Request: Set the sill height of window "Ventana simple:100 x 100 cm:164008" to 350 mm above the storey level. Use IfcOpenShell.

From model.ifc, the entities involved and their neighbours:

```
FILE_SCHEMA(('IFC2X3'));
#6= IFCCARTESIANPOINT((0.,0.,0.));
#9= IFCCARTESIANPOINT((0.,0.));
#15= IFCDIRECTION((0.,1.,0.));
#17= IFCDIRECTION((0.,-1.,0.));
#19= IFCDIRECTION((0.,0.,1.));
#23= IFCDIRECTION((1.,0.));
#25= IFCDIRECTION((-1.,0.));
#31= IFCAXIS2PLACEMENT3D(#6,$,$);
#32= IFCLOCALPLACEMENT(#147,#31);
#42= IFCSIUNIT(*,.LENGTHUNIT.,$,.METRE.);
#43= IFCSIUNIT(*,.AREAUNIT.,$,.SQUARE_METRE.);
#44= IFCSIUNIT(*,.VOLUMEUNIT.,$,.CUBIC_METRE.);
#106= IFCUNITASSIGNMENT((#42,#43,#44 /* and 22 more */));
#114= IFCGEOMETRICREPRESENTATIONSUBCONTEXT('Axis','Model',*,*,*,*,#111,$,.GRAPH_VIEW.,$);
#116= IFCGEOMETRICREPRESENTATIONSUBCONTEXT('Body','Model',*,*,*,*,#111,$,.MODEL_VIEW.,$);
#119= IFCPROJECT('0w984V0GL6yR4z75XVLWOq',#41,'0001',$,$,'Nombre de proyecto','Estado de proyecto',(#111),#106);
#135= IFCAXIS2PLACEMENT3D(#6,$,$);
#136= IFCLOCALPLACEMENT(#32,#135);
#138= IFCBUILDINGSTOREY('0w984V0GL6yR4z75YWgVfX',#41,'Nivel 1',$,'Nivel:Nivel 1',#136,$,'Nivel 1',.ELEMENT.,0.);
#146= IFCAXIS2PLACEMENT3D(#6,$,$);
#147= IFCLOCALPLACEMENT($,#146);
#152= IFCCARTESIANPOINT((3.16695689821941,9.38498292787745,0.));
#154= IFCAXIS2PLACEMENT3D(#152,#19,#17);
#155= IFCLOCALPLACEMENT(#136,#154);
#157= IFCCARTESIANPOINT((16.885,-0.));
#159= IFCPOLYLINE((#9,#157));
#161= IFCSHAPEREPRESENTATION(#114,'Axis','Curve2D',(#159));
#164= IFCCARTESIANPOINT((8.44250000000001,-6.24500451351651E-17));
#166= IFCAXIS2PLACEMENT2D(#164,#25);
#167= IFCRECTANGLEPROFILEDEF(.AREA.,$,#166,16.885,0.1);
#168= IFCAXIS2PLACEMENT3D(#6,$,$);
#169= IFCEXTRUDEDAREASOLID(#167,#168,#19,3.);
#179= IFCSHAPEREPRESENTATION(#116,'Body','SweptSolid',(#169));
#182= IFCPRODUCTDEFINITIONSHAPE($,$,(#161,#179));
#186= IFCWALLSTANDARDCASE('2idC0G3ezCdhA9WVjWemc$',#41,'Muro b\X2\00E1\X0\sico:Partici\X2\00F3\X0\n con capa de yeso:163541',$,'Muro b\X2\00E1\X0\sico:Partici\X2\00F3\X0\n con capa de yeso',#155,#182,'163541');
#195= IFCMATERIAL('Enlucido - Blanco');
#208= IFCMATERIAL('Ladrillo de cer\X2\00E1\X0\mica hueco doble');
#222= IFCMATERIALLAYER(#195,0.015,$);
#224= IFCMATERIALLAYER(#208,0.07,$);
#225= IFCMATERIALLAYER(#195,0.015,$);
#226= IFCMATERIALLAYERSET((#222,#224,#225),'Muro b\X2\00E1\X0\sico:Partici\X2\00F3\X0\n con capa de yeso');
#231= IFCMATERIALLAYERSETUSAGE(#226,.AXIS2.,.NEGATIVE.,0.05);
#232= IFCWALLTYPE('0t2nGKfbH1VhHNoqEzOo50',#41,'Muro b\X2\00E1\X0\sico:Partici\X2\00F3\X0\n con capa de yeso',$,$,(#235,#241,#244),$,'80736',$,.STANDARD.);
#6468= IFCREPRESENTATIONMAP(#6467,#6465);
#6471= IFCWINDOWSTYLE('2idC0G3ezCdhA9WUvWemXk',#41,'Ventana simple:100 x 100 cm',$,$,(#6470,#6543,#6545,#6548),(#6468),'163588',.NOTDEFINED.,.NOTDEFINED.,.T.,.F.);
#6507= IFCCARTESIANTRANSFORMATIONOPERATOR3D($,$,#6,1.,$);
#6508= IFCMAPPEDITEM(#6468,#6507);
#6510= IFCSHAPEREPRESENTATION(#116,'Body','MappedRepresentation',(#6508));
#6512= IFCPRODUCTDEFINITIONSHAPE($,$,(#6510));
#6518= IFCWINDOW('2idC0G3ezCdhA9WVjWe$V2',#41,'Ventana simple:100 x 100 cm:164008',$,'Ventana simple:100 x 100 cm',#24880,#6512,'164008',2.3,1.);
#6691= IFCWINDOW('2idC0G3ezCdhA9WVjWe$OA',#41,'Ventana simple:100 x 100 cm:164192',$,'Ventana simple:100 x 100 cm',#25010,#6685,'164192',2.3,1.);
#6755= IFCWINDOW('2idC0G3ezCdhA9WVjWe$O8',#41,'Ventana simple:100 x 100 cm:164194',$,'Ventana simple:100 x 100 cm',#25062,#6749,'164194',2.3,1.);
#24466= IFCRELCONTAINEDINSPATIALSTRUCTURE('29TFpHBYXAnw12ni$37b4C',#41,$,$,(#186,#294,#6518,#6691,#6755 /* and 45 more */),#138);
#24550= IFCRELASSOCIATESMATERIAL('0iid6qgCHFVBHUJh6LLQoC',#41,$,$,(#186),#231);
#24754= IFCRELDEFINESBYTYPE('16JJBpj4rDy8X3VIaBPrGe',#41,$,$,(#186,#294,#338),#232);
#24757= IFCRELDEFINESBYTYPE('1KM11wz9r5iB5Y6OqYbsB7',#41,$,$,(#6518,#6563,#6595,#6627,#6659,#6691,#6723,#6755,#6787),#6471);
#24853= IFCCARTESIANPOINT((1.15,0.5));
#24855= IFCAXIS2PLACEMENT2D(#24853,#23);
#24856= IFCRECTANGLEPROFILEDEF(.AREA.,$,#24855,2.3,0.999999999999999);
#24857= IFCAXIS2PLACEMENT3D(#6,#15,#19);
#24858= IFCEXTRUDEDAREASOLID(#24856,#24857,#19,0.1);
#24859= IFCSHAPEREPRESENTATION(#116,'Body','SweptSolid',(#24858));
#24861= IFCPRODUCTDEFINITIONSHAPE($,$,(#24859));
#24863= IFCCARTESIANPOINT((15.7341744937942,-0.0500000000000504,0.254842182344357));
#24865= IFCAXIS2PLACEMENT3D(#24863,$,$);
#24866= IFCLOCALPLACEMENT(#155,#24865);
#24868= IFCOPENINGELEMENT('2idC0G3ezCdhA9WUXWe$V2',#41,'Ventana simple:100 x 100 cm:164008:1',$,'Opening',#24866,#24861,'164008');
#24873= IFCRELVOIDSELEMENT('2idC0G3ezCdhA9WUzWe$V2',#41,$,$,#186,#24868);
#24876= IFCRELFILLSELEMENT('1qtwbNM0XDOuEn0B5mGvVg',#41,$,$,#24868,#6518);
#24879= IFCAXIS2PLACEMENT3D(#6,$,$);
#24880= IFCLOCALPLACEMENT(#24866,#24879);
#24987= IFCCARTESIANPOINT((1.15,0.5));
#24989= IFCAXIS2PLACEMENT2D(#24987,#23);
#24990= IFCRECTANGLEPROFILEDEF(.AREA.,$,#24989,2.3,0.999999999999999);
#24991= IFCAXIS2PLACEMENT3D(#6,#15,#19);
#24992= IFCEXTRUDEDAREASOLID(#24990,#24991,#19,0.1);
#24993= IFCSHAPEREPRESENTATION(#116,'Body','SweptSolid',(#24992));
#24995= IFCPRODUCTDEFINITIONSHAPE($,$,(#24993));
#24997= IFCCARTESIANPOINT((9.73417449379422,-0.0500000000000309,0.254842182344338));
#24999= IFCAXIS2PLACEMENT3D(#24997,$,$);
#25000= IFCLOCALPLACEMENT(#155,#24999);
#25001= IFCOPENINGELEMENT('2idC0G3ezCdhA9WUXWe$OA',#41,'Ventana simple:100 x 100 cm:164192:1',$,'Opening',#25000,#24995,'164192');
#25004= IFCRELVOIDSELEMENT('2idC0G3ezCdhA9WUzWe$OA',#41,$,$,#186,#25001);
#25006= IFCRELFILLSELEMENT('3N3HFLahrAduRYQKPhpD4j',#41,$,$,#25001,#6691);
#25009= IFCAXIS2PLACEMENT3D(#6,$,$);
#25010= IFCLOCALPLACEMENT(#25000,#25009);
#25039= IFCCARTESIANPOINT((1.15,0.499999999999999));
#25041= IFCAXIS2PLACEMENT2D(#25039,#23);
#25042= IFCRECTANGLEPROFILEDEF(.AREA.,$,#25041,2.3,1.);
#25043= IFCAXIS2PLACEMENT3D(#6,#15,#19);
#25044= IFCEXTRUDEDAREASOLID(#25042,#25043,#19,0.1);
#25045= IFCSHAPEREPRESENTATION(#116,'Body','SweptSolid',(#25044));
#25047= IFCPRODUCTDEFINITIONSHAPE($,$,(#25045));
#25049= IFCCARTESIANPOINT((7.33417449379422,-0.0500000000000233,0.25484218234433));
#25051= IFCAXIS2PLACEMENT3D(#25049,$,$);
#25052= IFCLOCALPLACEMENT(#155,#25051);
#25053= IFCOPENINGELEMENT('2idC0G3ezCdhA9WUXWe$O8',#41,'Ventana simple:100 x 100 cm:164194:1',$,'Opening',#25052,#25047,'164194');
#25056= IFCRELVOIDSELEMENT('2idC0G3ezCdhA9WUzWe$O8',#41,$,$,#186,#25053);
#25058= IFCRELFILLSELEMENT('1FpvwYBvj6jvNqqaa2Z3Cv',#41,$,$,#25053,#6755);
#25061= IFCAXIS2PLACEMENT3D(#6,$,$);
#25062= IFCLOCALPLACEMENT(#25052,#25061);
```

```python
import numpy as np
import ifcopenshell
import ifcopenshell.api.geometry
import ifcopenshell.geom
import ifcopenshell.util.element
import ifcopenshell.util.placement
import ifcopenshell.util.shape
import ifcopenshell.util.unit

model = ifcopenshell.open("model.ifc")
unit_scale = ifcopenshell.util.unit.calculate_unit_scale(model)

window = model.by_guid("2idC0G3ezCdhA9WVjWe$V2")
opening = window.FillsVoids[0].RelatingOpeningElement
storey = ifcopenshell.util.element.get_container(window, ifc_class="IfcBuildingStorey")
level = ifcopenshell.util.placement.get_local_placement(storey.ObjectPlacement)[2, 3]

# The opening's origin need not be at the sill, so measure its lowest point.
shape = ifcopenshell.geom.create_shape(ifcopenshell.geom.settings(), opening)
bottom = ifcopenshell.util.shape.get_shape_bottom_elevation(shape, shape.geometry) / unit_scale
dz = level + 0.35 / unit_scale - bottom

shift = np.array([0.0, 0.0, dz])
# The window is placed relative to its opening, so it follows when the opening moves.
matrix = ifcopenshell.util.placement.get_local_placement(opening.ObjectPlacement)
matrix[:3, 3] += shift
ifcopenshell.api.geometry.edit_object_placement(
    model, product=opening, matrix=matrix, is_si=False, should_transform_children=True
)

print(f"moved by {dz * unit_scale:+.3f} m")

model.write("model_edited.ifc")
```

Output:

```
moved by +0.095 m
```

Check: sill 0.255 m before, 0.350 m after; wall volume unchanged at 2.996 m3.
